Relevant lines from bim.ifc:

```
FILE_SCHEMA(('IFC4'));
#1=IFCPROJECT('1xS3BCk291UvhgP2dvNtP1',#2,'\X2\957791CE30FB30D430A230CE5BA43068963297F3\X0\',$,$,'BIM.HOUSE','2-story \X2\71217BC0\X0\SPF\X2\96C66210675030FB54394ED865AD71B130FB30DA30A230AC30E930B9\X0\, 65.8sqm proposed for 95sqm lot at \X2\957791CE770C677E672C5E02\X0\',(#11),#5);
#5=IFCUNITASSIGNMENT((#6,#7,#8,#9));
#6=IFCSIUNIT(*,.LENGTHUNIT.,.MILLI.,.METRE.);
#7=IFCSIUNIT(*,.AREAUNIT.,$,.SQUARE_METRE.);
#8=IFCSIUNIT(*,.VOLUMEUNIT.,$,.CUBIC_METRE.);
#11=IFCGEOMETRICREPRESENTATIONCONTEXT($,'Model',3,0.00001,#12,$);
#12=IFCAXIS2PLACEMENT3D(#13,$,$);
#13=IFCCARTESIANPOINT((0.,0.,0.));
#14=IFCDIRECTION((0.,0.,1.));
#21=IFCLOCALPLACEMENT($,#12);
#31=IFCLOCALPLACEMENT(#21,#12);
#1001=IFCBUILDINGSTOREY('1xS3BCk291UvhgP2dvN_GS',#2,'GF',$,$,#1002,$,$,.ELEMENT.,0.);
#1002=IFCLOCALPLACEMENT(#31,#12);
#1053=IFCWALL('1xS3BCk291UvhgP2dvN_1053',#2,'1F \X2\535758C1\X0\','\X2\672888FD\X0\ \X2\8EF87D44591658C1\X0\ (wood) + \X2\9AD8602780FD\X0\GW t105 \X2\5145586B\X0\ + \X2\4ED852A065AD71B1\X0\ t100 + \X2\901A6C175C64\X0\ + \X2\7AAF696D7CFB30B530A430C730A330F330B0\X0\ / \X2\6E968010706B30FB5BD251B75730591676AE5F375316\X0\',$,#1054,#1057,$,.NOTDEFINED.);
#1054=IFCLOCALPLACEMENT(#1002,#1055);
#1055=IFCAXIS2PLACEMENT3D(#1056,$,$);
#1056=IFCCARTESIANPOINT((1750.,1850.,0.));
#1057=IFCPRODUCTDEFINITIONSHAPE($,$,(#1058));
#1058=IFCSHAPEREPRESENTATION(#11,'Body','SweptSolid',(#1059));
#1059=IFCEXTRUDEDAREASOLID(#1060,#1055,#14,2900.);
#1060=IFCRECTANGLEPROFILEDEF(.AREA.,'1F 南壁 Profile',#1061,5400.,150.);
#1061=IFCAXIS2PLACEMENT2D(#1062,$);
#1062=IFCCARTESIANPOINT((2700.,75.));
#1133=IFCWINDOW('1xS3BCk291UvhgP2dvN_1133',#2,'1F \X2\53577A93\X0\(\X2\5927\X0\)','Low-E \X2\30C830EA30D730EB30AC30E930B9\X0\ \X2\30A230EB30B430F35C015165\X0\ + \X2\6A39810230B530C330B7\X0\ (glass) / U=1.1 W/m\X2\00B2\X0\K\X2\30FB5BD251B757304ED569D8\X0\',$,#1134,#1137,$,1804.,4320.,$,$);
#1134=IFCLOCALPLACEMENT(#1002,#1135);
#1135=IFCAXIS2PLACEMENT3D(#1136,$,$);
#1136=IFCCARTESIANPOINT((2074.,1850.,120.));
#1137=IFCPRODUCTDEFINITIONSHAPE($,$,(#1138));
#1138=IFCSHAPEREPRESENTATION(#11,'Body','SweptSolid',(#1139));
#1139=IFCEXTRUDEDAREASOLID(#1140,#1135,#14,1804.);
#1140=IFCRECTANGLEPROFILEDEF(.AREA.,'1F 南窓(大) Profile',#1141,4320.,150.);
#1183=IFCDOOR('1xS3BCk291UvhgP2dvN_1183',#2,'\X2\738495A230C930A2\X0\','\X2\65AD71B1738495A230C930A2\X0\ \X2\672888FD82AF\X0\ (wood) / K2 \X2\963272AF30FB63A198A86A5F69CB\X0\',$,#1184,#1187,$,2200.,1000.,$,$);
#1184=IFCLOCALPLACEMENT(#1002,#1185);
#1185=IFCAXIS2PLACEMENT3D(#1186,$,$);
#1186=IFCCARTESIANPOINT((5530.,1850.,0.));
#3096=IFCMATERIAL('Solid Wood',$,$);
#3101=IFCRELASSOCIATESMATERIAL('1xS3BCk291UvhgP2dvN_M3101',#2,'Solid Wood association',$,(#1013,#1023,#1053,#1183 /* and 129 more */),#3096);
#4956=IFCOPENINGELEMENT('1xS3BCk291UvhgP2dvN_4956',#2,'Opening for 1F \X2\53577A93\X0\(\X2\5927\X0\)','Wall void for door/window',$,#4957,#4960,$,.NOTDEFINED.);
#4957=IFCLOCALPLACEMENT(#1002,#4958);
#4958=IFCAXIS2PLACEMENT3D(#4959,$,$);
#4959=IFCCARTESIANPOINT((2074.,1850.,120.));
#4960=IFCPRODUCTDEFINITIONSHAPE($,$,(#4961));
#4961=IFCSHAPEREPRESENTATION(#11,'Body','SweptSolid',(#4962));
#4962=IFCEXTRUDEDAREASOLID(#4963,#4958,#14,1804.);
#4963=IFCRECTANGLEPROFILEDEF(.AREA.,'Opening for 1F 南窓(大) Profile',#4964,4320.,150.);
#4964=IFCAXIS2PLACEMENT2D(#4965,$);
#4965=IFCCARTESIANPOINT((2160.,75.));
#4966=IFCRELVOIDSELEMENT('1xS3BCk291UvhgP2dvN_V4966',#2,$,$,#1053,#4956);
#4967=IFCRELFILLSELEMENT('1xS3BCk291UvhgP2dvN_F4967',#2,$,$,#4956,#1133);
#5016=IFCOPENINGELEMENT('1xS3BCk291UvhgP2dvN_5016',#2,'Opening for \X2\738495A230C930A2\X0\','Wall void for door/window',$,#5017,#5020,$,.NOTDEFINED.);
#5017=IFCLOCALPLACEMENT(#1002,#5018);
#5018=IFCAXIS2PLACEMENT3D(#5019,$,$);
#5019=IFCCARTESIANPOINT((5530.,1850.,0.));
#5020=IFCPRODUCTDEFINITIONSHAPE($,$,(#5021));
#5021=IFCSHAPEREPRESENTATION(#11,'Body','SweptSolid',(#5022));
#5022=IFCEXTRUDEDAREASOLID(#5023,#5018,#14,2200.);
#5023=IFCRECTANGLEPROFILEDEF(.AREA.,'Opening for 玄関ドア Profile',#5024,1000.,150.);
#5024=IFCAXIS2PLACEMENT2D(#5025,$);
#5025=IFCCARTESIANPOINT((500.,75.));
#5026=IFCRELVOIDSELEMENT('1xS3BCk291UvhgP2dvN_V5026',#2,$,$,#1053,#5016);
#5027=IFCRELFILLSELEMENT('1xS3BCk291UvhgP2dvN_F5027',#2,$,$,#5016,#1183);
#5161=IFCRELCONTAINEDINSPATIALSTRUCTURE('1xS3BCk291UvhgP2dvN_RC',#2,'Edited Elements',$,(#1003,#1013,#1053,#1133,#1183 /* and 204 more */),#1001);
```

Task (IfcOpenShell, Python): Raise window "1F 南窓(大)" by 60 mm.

```python
import numpy as np
import ifcopenshell
import ifcopenshell.api.geometry
import ifcopenshell.util.placement
import ifcopenshell.util.unit

model = ifcopenshell.open("bim.ifc")
unit_scale = ifcopenshell.util.unit.calculate_unit_scale(model)

window = model.by_id(1133)
opening = window.FillsVoids[0].RelatingOpeningElement
dz = 0.06 / unit_scale

shift = np.array([0.0, 0.0, dz])
# The window is not placed relative to its opening, so move both.
for product in (opening, window):
    matrix = ifcopenshell.util.placement.get_local_placement(product.ObjectPlacement)
    matrix[:3, 3] += shift
    ifcopenshell.api.geometry.edit_object_placement(model, product=product, matrix=matrix, is_si=False)

print(f"moved by {dz * unit_scale:+.3f} m")

model.write("bim_updated.ifc")
```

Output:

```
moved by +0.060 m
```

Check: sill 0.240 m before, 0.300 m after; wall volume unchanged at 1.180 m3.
